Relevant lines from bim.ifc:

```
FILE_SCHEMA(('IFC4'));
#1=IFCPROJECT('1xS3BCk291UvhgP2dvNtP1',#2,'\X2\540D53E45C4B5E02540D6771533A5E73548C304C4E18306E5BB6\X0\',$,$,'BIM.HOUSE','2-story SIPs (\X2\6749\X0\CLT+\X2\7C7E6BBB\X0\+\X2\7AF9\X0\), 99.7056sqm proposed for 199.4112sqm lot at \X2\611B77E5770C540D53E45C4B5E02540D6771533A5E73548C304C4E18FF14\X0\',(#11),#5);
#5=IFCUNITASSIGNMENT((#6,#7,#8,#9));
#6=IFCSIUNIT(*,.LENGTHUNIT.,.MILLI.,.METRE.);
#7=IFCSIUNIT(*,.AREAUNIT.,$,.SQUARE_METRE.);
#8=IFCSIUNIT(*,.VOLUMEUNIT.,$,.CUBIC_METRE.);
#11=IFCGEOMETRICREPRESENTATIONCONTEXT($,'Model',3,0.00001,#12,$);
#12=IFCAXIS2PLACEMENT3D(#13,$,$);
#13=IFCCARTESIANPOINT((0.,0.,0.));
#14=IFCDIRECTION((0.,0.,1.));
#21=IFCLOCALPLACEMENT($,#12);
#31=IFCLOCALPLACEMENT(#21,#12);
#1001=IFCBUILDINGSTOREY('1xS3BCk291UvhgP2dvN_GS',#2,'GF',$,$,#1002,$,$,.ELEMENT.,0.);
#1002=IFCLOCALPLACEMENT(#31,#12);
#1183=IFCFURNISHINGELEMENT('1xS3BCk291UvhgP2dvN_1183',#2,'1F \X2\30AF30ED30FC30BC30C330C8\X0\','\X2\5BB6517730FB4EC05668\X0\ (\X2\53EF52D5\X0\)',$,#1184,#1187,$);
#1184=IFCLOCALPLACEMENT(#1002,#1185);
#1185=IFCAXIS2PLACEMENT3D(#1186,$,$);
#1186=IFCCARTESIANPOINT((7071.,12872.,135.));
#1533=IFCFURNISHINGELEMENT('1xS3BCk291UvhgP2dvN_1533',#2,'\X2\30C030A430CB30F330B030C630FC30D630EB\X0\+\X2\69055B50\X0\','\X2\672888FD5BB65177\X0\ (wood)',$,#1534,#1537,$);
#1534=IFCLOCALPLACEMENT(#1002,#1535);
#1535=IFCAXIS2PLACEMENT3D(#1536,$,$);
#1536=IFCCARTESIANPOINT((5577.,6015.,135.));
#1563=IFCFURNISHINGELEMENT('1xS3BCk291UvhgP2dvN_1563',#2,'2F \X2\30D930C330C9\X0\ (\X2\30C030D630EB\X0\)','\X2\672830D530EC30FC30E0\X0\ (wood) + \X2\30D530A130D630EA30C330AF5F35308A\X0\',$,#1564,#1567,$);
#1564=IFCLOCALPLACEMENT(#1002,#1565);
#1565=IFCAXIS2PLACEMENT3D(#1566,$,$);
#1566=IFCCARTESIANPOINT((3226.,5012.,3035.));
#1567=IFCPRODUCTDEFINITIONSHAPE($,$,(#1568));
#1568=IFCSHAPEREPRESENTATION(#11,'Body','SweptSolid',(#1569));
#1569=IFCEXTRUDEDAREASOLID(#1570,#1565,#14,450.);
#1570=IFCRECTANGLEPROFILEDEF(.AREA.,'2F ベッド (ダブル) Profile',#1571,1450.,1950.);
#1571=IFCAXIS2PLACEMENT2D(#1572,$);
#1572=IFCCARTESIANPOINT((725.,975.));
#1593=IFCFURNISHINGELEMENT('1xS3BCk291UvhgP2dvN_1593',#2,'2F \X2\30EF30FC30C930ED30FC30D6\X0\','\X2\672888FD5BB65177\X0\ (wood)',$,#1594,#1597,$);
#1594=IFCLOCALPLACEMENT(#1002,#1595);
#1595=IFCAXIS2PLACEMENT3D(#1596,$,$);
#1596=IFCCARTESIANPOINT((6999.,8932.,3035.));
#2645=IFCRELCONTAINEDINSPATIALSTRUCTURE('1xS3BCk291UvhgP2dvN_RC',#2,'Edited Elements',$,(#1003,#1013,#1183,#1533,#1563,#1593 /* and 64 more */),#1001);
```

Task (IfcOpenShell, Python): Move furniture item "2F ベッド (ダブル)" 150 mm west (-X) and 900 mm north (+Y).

```python
import ifcopenshell
import ifcopenshell.api.geometry
import ifcopenshell.util.placement

model = ifcopenshell.open("bim.ifc")

item = model.by_guid("1xS3BCk291UvhgP2dvN_1563")
matrix = ifcopenshell.util.placement.get_local_placement(item.ObjectPlacement)
matrix[0, 3] -= 150.0
matrix[1, 3] += 900.0
ifcopenshell.api.geometry.edit_object_placement(model, product=item, matrix=matrix, is_si=False)

print(ifcopenshell.util.placement.get_local_placement(item.ObjectPlacement).round(3) + 0.0)

model.write("bim_v2.ifc")
```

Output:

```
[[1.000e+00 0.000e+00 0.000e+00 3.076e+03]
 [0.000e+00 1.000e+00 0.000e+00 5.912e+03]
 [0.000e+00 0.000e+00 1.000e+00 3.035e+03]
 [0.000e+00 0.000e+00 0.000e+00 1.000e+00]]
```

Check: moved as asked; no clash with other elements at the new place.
